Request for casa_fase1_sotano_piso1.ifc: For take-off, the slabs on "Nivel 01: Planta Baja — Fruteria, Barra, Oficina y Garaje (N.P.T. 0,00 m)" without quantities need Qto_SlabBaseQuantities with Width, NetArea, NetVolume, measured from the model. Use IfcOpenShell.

First a look at what the model holds.

```python
import ifcopenshell
import ifcopenshell.util.element
import ifcopenshell.util.unit

model = ifcopenshell.open("casa_fase1_sotano_piso1.ifc")
print(model.schema)
for unit_type in ("LENGTHUNIT", "AREAUNIT", "VOLUMEUNIT"):
    print(unit_type, ifcopenshell.util.unit.calculate_unit_scale(model, unit_type))
storey = next(s for s in model.by_type("IfcBuildingStorey") if s.Name == "Nivel 01: Planta Baja — Fruteria, Barra, Oficina y Garaje (N.P.T. 0,00 m)")
slabs = [e for e in ifcopenshell.util.element.get_decomposition(storey) if e.is_a("IfcSlab")]
for e in sorted(slabs, key=lambda e: e.id()):
    print(e.id(), e.is_a(), e.Name, list(ifcopenshell.util.element.get_psets(e, qtos_only=True)), sep=" | ")
```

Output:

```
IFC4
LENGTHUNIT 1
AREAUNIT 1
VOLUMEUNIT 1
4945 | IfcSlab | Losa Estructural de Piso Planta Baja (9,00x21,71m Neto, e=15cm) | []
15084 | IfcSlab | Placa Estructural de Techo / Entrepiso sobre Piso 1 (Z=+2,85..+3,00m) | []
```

```python
import ifcopenshell
import ifcopenshell.api.pset
import ifcopenshell.geom
import ifcopenshell.util.element
import ifcopenshell.util.shape
import ifcopenshell.util.unit

model = ifcopenshell.open("casa_fase1_sotano_piso1.ifc")
unit_scale = ifcopenshell.util.unit.calculate_unit_scale(model)
area_scale = ifcopenshell.util.unit.calculate_unit_scale(model, "AREAUNIT")
volume_scale = ifcopenshell.util.unit.calculate_unit_scale(model, "VOLUMEUNIT")
settings = ifcopenshell.geom.settings()

storey = next(s for s in model.by_type("IfcBuildingStorey") if s.Name == "Nivel 01: Planta Baja — Fruteria, Barra, Oficina y Garaje (N.P.T. 0,00 m)")
slabs = [e for e in ifcopenshell.util.element.get_decomposition(storey) if e.is_a("IfcSlab")]

for e in sorted(slabs, key=lambda e: e.id()):
    if ifcopenshell.util.element.get_psets(e, qtos_only=True, should_inherit=False):
        continue
    # Geometry comes back in metres, in the element's own axes.
    shape = ifcopenshell.geom.create_shape(settings, e)
    values = {
        "Width": ifcopenshell.util.shape.get_z(shape.geometry) / unit_scale,
        "NetArea": ifcopenshell.util.shape.get_footprint_area(shape.geometry) / area_scale,
        "NetVolume": ifcopenshell.util.shape.get_volume(shape.geometry) / volume_scale,
    }
    qto = ifcopenshell.api.pset.add_qto(model, product=e, name="Qto_SlabBaseQuantities")
    ifcopenshell.api.pset.edit_qto(model, qto=qto, properties=values)
    print(e.id(), {k: round(v, 3) for k, v in values.items()})

model.write("casa_fase1_sotano_piso1_updated.ifc")
```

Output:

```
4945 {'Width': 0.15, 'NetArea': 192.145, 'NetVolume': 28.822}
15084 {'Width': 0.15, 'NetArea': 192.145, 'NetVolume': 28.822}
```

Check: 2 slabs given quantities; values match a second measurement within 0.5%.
